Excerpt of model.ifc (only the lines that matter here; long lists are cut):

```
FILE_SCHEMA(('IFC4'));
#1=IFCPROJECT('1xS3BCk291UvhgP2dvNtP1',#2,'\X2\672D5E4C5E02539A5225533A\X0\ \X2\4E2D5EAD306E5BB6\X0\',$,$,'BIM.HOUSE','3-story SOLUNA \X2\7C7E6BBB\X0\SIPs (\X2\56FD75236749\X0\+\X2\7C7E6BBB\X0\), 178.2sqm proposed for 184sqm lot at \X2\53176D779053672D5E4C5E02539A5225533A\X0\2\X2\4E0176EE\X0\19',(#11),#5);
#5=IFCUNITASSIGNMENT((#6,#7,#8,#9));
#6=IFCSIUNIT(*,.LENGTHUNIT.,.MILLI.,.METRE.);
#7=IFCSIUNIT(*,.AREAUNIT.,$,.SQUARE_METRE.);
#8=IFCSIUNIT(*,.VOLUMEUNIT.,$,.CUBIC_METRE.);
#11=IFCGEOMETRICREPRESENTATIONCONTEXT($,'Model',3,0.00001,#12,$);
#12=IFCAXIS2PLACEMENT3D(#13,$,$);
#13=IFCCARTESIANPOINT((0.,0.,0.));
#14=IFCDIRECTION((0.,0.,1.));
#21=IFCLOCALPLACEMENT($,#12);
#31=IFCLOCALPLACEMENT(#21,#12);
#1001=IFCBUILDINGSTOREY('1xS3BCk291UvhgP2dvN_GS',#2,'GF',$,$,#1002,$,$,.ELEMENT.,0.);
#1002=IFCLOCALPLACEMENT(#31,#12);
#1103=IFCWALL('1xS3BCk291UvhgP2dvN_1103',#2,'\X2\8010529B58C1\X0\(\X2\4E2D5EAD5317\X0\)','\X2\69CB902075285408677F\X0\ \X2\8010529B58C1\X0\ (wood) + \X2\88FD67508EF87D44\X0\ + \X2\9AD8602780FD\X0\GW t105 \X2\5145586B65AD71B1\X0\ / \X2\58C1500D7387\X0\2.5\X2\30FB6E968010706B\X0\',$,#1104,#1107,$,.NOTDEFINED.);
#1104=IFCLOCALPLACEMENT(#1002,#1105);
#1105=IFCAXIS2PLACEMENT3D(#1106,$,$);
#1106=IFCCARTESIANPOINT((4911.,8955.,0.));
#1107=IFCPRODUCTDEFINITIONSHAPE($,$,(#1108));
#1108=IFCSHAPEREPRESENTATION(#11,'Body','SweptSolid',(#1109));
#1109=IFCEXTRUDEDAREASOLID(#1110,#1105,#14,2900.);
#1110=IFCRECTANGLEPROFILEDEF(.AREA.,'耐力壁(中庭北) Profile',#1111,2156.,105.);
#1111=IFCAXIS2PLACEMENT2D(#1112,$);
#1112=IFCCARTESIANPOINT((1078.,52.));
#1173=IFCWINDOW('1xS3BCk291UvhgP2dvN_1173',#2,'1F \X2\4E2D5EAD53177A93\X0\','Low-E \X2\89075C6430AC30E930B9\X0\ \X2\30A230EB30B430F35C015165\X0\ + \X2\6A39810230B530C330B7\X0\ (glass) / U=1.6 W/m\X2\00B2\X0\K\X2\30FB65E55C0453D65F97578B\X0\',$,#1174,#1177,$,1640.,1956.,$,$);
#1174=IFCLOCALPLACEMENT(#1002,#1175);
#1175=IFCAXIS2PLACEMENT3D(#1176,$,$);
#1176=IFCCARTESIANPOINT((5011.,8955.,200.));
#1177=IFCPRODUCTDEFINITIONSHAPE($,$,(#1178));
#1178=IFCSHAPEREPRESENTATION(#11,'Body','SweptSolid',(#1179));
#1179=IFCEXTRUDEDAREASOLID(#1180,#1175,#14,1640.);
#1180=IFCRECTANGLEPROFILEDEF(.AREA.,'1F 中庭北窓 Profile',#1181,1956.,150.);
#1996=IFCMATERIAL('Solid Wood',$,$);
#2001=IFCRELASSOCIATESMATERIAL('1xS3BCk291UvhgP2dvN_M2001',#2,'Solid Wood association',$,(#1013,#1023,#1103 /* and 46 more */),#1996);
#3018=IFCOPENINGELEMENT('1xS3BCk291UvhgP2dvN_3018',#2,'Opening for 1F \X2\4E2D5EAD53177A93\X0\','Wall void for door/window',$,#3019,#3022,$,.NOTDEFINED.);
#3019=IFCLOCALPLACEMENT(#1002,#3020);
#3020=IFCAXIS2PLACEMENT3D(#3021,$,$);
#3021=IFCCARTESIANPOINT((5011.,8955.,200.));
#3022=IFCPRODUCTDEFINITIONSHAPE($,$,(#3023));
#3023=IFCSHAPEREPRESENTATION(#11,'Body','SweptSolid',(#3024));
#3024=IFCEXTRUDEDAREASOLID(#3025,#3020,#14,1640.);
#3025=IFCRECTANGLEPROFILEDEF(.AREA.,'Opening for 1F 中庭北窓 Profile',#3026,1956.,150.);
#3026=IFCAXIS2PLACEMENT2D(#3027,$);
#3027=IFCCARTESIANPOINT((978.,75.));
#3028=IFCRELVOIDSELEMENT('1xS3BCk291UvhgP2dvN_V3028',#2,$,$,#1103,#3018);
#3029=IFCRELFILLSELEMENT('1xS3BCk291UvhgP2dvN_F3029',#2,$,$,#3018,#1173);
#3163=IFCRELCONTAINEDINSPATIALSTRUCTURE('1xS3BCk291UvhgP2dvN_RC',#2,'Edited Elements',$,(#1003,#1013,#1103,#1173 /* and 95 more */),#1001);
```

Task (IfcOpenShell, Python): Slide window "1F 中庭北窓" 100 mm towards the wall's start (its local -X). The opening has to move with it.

```python
import ifcopenshell
import ifcopenshell.api.geometry
import ifcopenshell.util.placement

model = ifcopenshell.open("model.ifc")

window = model.by_guid("1xS3BCk291UvhgP2dvN_1173")
opening = window.FillsVoids[0].RelatingOpeningElement
wall = opening.VoidsElements[0].RelatingBuildingElement

wall_matrix = ifcopenshell.util.placement.get_local_placement(wall.ObjectPlacement)
shift = wall_matrix[:3, 0] * -100.0
before = ifcopenshell.util.placement.get_local_placement(window.ObjectPlacement)[:3, 3].copy()

# The window is not placed relative to its opening, so move both.
for product in (opening, window):
    matrix = ifcopenshell.util.placement.get_local_placement(product.ObjectPlacement)
    matrix[:3, 3] += shift
    ifcopenshell.api.geometry.edit_object_placement(model, product=product, matrix=matrix, is_si=False)

after = ifcopenshell.util.placement.get_local_placement(window.ObjectPlacement)[:3, 3]
print("window moved by", (after - before).round(3) + 0.0)

model.write("model_rev.ifc")
```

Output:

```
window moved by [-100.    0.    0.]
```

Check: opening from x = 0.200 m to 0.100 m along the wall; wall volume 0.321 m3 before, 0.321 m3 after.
